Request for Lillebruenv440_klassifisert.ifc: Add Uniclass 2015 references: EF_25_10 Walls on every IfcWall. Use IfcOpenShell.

First a look at what the model holds.

```python
import ifcopenshell

model = ifcopenshell.open("Lillebruenv440_klassifisert.ifc")
print(model.schema)
print("classifications:", [c.Name for c in model.by_type("IfcClassification")])
for ifc_class in ("IfcDoor", "IfcRoof", "IfcStair", "IfcWall", "IfcWindow"):
    print(ifc_class, len(model.by_type(ifc_class)))
```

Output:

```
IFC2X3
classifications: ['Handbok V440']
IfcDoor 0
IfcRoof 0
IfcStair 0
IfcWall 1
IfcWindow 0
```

```python
import ifcopenshell
import ifcopenshell.api.classification

model = ifcopenshell.open("Lillebruenv440_klassifisert.ifc")

# IFC2X3 requires Source and Edition and has no link from the project to the system.
system = model.create_entity("IfcClassification", Source="NBS", Edition="2015", Name="Uniclass 2015")

codes = {
    "IfcWall": ("EF_25_10", "Walls"),
}
for ifc_class, (code, name) in codes.items():
    products = model.by_type(ifc_class)
    ifcopenshell.api.classification.add_reference(
        model, products=products, classification=system, identification=code, name=name
    )
    print(code, len(products))

model.write("Lillebruenv440_klassifisert_updated.ifc")
```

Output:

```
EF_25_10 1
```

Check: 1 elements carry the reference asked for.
